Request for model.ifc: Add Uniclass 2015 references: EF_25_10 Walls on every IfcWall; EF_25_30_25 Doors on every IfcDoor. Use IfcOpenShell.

First a look at what the model holds.

```python
import ifcopenshell

model = ifcopenshell.open("model.ifc")
print(model.schema)
print("classifications:", [c.Name for c in model.by_type("IfcClassification")])
for ifc_class in ("IfcDoor", "IfcRoof", "IfcStair", "IfcWall", "IfcWindow"):
    print(ifc_class, len(model.by_type(ifc_class)))
```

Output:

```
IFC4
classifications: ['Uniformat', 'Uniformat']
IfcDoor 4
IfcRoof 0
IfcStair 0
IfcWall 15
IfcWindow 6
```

```python
import ifcopenshell
import ifcopenshell.api.classification

model = ifcopenshell.open("model.ifc")

system = ifcopenshell.api.classification.add_classification(model, classification="Uniclass 2015")

codes = {
    "IfcWall": ("EF_25_10", "Walls"),
    "IfcDoor": ("EF_25_30_25", "Doors"),
}
for ifc_class, (code, name) in codes.items():
    products = model.by_type(ifc_class)
    ifcopenshell.api.classification.add_reference(
        model, products=products, classification=system, identification=code, name=name
    )
    print(code, len(products))

model.write("model_rev.ifc")
```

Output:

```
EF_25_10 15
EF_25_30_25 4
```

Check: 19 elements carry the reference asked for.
